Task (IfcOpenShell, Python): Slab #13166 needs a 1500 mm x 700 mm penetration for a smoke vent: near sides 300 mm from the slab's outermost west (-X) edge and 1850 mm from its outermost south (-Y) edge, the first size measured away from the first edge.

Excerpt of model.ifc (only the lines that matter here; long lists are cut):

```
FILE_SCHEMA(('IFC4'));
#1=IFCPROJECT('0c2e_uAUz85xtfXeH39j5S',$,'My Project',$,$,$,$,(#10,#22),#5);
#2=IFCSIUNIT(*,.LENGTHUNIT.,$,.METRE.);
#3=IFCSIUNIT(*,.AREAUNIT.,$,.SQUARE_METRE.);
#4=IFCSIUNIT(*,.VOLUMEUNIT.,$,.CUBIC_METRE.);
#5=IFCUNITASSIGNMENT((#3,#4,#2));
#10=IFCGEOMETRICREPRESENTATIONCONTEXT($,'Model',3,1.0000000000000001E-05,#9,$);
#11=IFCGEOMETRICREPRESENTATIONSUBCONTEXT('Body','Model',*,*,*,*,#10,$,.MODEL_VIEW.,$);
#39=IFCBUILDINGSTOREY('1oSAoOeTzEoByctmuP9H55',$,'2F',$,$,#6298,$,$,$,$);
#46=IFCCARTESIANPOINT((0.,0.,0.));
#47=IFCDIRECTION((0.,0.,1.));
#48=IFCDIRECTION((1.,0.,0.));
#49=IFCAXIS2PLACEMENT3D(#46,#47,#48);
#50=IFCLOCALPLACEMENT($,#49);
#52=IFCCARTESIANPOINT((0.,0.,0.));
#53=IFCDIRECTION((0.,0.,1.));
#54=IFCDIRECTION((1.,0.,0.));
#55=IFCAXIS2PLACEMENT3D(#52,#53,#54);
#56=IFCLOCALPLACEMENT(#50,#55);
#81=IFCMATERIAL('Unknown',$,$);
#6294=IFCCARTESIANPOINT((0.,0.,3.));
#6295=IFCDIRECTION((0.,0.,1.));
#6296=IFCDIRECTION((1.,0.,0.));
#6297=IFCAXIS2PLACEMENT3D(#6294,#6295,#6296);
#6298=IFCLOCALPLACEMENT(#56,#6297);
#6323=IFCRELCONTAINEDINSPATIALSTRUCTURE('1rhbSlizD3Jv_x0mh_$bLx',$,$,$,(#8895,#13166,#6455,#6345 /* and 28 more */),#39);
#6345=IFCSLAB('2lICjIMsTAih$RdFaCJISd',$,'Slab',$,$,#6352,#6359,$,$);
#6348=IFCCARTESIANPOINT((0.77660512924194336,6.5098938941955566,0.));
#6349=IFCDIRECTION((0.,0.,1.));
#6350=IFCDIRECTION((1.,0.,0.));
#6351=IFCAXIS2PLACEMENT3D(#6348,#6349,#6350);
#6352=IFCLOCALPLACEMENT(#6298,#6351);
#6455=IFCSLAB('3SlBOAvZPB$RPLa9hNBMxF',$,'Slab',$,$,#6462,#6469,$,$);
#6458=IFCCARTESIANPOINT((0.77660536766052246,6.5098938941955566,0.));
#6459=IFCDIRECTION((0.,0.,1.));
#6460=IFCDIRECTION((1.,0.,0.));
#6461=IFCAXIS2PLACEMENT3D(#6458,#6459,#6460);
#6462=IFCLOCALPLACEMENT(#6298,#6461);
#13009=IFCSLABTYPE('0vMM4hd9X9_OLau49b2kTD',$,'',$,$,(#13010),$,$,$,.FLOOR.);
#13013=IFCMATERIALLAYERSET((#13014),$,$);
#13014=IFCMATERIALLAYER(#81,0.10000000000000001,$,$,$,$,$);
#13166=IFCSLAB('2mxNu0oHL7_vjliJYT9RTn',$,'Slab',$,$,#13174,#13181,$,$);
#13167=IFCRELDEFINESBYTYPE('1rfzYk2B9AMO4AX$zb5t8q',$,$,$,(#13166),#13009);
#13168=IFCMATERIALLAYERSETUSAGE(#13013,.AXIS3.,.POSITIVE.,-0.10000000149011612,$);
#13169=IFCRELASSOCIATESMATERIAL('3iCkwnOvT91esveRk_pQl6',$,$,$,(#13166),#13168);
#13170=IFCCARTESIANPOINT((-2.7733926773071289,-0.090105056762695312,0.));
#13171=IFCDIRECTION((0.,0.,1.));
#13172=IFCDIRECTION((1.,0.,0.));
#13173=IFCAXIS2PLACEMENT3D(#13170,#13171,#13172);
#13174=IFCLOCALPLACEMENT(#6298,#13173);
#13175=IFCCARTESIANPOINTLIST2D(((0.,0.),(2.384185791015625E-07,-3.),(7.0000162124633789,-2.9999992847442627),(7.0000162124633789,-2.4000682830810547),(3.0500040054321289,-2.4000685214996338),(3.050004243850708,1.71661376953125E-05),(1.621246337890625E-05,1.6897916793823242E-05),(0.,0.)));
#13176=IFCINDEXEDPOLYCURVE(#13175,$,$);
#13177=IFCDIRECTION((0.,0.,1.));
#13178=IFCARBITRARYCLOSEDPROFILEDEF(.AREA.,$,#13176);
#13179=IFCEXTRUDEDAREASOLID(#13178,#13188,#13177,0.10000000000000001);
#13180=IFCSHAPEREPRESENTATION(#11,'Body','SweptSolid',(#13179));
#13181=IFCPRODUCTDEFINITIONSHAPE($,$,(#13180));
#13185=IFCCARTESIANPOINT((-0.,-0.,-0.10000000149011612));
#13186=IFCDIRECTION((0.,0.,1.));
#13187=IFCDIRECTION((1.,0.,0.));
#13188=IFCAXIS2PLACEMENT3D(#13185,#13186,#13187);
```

```python
import numpy as np
import ifcopenshell
import ifcopenshell.api.feature
import ifcopenshell.api.geometry
import ifcopenshell.api.root
import ifcopenshell.geom
import ifcopenshell.util.placement
import ifcopenshell.util.representation
import ifcopenshell.util.shape
import ifcopenshell.util.unit

model = ifcopenshell.open("model.ifc")
unit_scale = ifcopenshell.util.unit.calculate_unit_scale(model)
settings = ifcopenshell.geom.settings()


def volume(element):
    """Net volume in cubic metres, openings subtracted."""
    shape = ifcopenshell.geom.create_shape(settings, element)
    return ifcopenshell.util.shape.get_volume(shape.geometry)


slab = model.by_id(13166)
before = volume(slab)

# Extent in the slab's own axes, in metres. The edges named are its -X and -Y sides.
slab_shape = ifcopenshell.geom.create_shape(settings, slab)
vertices = ifcopenshell.util.shape.get_vertices(slab_shape.geometry)
x_min, y_min, bottom = vertices.min(axis=0)
top = vertices[:, 2].max()

opening = ifcopenshell.api.root.create_entity(model, ifc_class="IfcOpeningElement", name="Smoke vent opening", predefined_type="OPENING")
context = ifcopenshell.util.representation.get_context(model, "Model", "Body", "MODEL_VIEW")
width, depth = 1.5, 0.7
outline = [(0.0, 0.0), (width, 0.0), (width, depth), (0.0, depth), (0.0, 0.0)]
# Overshoot both faces by 50 mm so the cut is clean.
shape = ifcopenshell.api.geometry.add_slab_representation(
    model, context=context, depth=top - bottom + 0.1, polyline=outline
)
ifcopenshell.api.geometry.assign_representation(model, product=opening, representation=shape)

matrix = ifcopenshell.util.placement.get_local_placement(slab.ObjectPlacement)
matrix[:, 3] = matrix @ np.append(np.array([x_min + 0.3, y_min + 1.85, bottom - 0.05]) / unit_scale, 1.0)
ifcopenshell.api.geometry.edit_object_placement(model, product=opening, matrix=matrix, is_si=False)
ifcopenshell.api.feature.add_feature(model, feature=opening, element=slab)

after = volume(slab)

print(f"slab volume {before:.3f} -> {after:.3f} m3")

model.write("model-out.ifc")
```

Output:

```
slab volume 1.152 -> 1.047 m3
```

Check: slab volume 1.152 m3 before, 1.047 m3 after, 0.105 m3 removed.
